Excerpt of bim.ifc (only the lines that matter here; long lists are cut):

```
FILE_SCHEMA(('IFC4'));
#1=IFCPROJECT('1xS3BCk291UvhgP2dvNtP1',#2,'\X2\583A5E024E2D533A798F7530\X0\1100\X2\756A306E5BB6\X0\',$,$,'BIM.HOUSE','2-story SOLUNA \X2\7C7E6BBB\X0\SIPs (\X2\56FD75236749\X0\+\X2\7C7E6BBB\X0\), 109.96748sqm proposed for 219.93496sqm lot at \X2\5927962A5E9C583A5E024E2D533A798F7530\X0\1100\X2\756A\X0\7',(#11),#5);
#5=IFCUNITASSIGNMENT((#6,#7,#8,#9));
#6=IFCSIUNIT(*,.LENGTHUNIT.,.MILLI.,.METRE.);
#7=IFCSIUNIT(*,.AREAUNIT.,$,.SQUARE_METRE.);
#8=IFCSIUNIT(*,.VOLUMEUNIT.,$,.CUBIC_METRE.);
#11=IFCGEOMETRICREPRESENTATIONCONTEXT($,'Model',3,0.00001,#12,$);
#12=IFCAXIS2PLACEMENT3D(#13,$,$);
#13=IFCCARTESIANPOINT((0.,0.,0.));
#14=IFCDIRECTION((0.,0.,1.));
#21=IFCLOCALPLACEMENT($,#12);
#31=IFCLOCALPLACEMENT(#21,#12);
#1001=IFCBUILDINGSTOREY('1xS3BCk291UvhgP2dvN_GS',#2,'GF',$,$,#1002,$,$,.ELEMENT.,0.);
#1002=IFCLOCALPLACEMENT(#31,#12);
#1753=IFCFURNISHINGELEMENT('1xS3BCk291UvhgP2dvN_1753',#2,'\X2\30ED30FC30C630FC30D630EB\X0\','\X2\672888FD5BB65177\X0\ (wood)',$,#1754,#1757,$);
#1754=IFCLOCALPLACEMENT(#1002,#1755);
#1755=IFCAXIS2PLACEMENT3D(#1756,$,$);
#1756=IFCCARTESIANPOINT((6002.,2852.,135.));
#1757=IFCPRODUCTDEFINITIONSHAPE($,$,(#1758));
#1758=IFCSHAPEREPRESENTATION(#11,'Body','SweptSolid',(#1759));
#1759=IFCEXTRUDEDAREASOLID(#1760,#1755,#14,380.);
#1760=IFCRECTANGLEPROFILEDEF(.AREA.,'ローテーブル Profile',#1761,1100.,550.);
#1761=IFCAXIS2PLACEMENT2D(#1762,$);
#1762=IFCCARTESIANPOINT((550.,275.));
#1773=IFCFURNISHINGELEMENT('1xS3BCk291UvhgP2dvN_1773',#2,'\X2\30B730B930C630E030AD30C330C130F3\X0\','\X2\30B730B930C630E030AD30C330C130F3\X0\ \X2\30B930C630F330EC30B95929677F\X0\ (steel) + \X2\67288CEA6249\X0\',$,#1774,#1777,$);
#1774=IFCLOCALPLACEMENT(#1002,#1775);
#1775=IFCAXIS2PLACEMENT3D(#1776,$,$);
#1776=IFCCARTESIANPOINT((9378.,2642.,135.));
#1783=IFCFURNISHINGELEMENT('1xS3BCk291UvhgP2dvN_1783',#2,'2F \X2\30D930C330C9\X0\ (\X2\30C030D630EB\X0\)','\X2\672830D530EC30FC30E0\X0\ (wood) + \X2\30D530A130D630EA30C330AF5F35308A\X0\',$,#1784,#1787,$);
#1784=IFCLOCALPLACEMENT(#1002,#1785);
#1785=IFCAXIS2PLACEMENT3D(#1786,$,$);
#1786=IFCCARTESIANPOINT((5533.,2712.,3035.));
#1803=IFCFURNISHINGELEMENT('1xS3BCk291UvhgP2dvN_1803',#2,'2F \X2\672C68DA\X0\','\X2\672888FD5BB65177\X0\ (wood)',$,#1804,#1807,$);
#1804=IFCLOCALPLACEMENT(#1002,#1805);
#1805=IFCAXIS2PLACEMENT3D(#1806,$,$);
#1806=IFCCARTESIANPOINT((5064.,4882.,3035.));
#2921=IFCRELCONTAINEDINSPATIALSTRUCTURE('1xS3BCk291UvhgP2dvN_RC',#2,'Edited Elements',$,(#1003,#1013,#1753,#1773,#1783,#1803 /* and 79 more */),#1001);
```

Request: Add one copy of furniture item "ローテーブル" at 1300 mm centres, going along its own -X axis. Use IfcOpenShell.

```python
import ifcopenshell
import ifcopenshell.api.geometry
import ifcopenshell.api.root
import ifcopenshell.util.element
import ifcopenshell.util.placement

model = ifcopenshell.open("bim.ifc")


def reuse_history(source, copy):
    """copy_class also copies each property set's owner history, people and application; keep the originals."""
    for rel in copy.IsDefinedBy:
        if rel.is_a("IfcRelDefinesByProperties") and (history := rel.RelatingPropertyDefinition.OwnerHistory):
            rel.RelatingPropertyDefinition.OwnerHistory = source.OwnerHistory
            ifcopenshell.util.element.remove_deep2(model, history)


source = model.by_guid("1xS3BCk291UvhgP2dvN_1753")
base = ifcopenshell.util.placement.get_local_placement(source.ObjectPlacement)
step = -base[:3, 0] * 1300.0

for i in range(1, 2):
    copy = ifcopenshell.api.root.copy_class(model, product=source)
    copy.Representation = ifcopenshell.util.element.copy_deep(
        model, source.Representation, exclude=["IfcGeometricRepresentationContext", "IfcRepresentationMap"]
    )
    reuse_history(source, copy)
    matrix = base.copy()
    matrix[:3, 3] += i * step
    print("added at", matrix[:3, 3].round(3) + 0.0)
    ifcopenshell.api.geometry.edit_object_placement(model, product=copy, matrix=matrix, is_si=False)

model.write("bim_rev.ifc")
```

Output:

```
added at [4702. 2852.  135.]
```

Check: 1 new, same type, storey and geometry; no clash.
